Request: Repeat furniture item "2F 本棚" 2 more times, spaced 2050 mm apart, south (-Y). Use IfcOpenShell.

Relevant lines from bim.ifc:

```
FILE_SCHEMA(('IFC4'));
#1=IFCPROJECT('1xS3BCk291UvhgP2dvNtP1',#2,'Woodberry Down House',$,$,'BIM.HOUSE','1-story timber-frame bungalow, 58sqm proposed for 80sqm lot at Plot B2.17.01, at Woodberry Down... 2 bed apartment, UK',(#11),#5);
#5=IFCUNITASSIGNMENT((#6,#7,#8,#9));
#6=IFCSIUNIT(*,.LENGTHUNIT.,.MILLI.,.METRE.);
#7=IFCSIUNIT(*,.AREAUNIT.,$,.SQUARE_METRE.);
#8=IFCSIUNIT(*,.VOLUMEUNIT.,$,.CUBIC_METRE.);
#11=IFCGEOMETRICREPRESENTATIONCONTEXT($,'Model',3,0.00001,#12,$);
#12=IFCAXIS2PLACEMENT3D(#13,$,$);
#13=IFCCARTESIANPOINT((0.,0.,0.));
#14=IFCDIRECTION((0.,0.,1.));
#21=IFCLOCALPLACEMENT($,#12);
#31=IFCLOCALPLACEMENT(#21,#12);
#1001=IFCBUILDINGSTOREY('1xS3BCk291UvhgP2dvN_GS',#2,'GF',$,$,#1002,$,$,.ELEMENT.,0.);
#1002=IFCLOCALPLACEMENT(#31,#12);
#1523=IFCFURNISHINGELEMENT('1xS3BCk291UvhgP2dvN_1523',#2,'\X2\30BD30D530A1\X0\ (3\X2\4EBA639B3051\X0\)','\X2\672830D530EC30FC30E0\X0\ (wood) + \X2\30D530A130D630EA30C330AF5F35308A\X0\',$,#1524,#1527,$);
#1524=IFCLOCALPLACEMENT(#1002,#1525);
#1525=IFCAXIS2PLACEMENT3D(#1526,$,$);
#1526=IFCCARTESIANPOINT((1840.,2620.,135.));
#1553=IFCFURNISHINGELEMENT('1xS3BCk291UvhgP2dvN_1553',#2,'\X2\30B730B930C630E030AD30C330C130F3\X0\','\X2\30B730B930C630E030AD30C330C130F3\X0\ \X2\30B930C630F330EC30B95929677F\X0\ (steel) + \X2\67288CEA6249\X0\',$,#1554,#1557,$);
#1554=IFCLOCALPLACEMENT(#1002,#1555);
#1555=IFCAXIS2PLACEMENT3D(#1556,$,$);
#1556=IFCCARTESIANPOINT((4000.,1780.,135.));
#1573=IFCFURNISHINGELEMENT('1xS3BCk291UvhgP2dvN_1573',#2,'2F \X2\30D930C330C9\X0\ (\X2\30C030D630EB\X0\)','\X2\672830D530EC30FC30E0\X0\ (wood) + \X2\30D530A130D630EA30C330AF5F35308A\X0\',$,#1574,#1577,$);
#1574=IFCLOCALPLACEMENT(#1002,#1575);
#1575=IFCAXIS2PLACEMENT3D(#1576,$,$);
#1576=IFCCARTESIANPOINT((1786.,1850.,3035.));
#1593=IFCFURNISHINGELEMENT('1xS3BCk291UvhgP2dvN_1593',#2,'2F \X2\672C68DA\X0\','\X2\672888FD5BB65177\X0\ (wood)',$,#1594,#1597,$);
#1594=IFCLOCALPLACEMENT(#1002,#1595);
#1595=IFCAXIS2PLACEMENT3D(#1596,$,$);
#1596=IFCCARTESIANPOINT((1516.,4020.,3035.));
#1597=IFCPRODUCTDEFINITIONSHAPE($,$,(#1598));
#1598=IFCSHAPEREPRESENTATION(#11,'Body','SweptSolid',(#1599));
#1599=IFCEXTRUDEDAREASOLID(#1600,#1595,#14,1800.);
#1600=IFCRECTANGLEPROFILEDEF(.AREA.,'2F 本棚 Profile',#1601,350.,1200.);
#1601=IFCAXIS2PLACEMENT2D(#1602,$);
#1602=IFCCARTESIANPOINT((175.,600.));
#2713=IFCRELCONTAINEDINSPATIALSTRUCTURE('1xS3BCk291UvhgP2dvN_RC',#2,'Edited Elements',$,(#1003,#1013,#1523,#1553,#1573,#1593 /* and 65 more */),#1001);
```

```python
import numpy as np
import ifcopenshell
import ifcopenshell.api.geometry
import ifcopenshell.api.root
import ifcopenshell.util.element
import ifcopenshell.util.placement
import ifcopenshell.util.unit

model = ifcopenshell.open("bim.ifc")
unit_scale = ifcopenshell.util.unit.calculate_unit_scale(model)


def reuse_history(source, copy):
    """copy_class also copies each property set's owner history, people and application; keep the originals."""
    for rel in copy.IsDefinedBy:
        if rel.is_a("IfcRelDefinesByProperties") and (history := rel.RelatingPropertyDefinition.OwnerHistory):
            rel.RelatingPropertyDefinition.OwnerHistory = source.OwnerHistory
            ifcopenshell.util.element.remove_deep2(model, history)


source = model.by_id(1593)
base = ifcopenshell.util.placement.get_local_placement(source.ObjectPlacement)
step = np.array([0.0, -1.0, 0.0]) * 2.05 / unit_scale

for i in range(1, 3):
    copy = ifcopenshell.api.root.copy_class(model, product=source)
    copy.Representation = ifcopenshell.util.element.copy_deep(
        model, source.Representation, exclude=["IfcGeometricRepresentationContext", "IfcRepresentationMap"]
    )
    reuse_history(source, copy)
    matrix = base.copy()
    matrix[:3, 3] += i * step
    print("added at", matrix[:3, 3].round(3) + 0.0)
    ifcopenshell.api.geometry.edit_object_placement(model, product=copy, matrix=matrix, is_si=False)

model.write("bim_v2.ifc")
```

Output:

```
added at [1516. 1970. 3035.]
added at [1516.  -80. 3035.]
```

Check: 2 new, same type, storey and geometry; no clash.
